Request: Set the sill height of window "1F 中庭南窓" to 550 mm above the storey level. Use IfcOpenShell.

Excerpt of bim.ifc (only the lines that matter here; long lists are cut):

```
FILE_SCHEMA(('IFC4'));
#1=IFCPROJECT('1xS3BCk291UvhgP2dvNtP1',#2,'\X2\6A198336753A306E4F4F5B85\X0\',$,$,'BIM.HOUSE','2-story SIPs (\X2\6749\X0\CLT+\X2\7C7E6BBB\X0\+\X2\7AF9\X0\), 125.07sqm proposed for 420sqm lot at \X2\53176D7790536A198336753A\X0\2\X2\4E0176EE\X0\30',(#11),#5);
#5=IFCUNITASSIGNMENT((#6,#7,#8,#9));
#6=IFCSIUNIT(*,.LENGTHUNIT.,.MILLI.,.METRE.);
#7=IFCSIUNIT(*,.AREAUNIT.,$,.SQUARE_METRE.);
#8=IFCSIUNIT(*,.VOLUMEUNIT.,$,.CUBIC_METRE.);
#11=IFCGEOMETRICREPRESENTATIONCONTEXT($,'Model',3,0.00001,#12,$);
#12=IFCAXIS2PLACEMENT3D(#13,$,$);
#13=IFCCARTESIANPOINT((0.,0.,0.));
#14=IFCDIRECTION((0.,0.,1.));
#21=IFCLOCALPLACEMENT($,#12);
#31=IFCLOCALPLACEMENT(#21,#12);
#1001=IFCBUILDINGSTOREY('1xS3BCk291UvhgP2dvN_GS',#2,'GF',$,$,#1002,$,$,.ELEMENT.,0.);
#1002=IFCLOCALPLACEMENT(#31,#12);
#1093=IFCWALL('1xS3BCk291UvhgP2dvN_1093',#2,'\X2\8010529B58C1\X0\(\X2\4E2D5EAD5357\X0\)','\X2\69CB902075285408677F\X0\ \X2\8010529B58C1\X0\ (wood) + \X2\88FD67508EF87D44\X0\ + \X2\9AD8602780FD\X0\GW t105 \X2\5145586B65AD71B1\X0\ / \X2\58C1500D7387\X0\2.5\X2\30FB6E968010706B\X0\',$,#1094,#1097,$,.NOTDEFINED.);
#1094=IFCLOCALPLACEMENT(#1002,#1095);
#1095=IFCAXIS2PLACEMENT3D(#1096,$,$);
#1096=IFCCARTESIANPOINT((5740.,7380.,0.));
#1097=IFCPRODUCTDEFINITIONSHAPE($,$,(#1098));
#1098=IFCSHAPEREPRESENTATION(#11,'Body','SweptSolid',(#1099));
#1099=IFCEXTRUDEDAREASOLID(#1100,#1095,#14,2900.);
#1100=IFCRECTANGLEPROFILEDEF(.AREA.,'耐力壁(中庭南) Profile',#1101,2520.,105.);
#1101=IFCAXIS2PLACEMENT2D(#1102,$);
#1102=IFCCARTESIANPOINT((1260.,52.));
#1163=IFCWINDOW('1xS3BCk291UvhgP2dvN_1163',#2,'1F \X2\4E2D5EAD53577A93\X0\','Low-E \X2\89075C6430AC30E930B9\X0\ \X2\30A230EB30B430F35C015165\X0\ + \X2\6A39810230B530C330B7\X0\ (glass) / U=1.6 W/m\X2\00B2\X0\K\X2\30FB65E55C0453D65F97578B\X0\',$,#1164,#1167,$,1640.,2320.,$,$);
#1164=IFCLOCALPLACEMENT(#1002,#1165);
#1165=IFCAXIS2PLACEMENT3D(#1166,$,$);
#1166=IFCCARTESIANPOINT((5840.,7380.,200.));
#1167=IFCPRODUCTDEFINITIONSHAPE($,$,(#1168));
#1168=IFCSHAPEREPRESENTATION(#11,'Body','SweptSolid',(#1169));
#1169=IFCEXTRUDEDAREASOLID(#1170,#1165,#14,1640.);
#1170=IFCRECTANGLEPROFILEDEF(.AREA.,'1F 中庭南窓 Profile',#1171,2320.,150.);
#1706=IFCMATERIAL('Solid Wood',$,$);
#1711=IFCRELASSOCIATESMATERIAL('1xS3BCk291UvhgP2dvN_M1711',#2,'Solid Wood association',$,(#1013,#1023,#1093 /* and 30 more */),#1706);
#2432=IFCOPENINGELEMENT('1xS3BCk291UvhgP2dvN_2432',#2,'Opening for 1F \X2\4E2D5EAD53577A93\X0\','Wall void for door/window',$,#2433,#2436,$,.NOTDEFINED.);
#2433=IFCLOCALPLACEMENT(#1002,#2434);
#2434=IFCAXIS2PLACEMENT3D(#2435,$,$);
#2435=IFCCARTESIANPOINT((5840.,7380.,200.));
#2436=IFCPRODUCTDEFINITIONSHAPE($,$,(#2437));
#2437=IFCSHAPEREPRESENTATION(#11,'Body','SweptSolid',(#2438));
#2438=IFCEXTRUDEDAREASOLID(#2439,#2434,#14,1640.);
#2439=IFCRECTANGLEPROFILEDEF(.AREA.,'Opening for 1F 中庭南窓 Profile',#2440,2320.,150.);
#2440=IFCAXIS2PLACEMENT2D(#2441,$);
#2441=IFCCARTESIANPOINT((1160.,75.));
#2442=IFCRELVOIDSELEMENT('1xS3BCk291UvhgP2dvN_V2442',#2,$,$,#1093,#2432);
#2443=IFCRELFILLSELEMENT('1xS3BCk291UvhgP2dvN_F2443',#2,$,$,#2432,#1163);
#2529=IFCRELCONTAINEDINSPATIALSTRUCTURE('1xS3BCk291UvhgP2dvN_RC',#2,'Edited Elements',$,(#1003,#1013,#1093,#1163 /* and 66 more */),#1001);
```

```python
import numpy as np
import ifcopenshell
import ifcopenshell.api.geometry
import ifcopenshell.geom
import ifcopenshell.util.element
import ifcopenshell.util.placement
import ifcopenshell.util.shape
import ifcopenshell.util.unit

model = ifcopenshell.open("bim.ifc")
unit_scale = ifcopenshell.util.unit.calculate_unit_scale(model)

window = model.by_guid("1xS3BCk291UvhgP2dvN_1163")
opening = window.FillsVoids[0].RelatingOpeningElement
storey = ifcopenshell.util.element.get_container(window, ifc_class="IfcBuildingStorey")
level = ifcopenshell.util.placement.get_local_placement(storey.ObjectPlacement)[2, 3]

# The opening's origin need not be at the sill, so measure its lowest point.
shape = ifcopenshell.geom.create_shape(ifcopenshell.geom.settings(), opening)
bottom = ifcopenshell.util.shape.get_shape_bottom_elevation(shape, shape.geometry) / unit_scale
dz = level + 550.0 - bottom

shift = np.array([0.0, 0.0, dz])
# The window is not placed relative to its opening, so move both.
for product in (opening, window):
    matrix = ifcopenshell.util.placement.get_local_placement(product.ObjectPlacement)
    matrix[:3, 3] += shift
    ifcopenshell.api.geometry.edit_object_placement(model, product=product, matrix=matrix, is_si=False)

print(f"moved by {dz * unit_scale:+.3f} m")

model.write("bim_rev.ifc")
```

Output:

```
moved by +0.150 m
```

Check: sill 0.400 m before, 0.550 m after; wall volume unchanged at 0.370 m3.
